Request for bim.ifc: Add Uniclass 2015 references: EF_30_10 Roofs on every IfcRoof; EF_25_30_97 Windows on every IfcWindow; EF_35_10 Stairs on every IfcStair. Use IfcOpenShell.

First a look at what the model holds.

```python
import ifcopenshell

model = ifcopenshell.open("bim.ifc")
print(model.schema)
print("classifications:", [c.Name for c in model.by_type("IfcClassification")])
for ifc_class in ("IfcDoor", "IfcRoof", "IfcStair", "IfcWall", "IfcWindow"):
    print(ifc_class, len(model.by_type(ifc_class)))
```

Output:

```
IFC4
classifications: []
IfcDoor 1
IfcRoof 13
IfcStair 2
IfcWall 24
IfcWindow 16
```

```python
import ifcopenshell
import ifcopenshell.api.classification

model = ifcopenshell.open("bim.ifc")

system = ifcopenshell.api.classification.add_classification(model, classification="Uniclass 2015")

codes = {
    "IfcRoof": ("EF_30_10", "Roofs"),
    "IfcWindow": ("EF_25_30_97", "Windows"),
    "IfcStair": ("EF_35_10", "Stairs"),
}
for ifc_class, (code, name) in codes.items():
    products = model.by_type(ifc_class)
    ifcopenshell.api.classification.add_reference(
        model, products=products, classification=system, identification=code, name=name
    )
    print(code, len(products))

model.write("bim_edited.ifc")
```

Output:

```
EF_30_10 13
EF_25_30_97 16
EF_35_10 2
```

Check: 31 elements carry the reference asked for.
